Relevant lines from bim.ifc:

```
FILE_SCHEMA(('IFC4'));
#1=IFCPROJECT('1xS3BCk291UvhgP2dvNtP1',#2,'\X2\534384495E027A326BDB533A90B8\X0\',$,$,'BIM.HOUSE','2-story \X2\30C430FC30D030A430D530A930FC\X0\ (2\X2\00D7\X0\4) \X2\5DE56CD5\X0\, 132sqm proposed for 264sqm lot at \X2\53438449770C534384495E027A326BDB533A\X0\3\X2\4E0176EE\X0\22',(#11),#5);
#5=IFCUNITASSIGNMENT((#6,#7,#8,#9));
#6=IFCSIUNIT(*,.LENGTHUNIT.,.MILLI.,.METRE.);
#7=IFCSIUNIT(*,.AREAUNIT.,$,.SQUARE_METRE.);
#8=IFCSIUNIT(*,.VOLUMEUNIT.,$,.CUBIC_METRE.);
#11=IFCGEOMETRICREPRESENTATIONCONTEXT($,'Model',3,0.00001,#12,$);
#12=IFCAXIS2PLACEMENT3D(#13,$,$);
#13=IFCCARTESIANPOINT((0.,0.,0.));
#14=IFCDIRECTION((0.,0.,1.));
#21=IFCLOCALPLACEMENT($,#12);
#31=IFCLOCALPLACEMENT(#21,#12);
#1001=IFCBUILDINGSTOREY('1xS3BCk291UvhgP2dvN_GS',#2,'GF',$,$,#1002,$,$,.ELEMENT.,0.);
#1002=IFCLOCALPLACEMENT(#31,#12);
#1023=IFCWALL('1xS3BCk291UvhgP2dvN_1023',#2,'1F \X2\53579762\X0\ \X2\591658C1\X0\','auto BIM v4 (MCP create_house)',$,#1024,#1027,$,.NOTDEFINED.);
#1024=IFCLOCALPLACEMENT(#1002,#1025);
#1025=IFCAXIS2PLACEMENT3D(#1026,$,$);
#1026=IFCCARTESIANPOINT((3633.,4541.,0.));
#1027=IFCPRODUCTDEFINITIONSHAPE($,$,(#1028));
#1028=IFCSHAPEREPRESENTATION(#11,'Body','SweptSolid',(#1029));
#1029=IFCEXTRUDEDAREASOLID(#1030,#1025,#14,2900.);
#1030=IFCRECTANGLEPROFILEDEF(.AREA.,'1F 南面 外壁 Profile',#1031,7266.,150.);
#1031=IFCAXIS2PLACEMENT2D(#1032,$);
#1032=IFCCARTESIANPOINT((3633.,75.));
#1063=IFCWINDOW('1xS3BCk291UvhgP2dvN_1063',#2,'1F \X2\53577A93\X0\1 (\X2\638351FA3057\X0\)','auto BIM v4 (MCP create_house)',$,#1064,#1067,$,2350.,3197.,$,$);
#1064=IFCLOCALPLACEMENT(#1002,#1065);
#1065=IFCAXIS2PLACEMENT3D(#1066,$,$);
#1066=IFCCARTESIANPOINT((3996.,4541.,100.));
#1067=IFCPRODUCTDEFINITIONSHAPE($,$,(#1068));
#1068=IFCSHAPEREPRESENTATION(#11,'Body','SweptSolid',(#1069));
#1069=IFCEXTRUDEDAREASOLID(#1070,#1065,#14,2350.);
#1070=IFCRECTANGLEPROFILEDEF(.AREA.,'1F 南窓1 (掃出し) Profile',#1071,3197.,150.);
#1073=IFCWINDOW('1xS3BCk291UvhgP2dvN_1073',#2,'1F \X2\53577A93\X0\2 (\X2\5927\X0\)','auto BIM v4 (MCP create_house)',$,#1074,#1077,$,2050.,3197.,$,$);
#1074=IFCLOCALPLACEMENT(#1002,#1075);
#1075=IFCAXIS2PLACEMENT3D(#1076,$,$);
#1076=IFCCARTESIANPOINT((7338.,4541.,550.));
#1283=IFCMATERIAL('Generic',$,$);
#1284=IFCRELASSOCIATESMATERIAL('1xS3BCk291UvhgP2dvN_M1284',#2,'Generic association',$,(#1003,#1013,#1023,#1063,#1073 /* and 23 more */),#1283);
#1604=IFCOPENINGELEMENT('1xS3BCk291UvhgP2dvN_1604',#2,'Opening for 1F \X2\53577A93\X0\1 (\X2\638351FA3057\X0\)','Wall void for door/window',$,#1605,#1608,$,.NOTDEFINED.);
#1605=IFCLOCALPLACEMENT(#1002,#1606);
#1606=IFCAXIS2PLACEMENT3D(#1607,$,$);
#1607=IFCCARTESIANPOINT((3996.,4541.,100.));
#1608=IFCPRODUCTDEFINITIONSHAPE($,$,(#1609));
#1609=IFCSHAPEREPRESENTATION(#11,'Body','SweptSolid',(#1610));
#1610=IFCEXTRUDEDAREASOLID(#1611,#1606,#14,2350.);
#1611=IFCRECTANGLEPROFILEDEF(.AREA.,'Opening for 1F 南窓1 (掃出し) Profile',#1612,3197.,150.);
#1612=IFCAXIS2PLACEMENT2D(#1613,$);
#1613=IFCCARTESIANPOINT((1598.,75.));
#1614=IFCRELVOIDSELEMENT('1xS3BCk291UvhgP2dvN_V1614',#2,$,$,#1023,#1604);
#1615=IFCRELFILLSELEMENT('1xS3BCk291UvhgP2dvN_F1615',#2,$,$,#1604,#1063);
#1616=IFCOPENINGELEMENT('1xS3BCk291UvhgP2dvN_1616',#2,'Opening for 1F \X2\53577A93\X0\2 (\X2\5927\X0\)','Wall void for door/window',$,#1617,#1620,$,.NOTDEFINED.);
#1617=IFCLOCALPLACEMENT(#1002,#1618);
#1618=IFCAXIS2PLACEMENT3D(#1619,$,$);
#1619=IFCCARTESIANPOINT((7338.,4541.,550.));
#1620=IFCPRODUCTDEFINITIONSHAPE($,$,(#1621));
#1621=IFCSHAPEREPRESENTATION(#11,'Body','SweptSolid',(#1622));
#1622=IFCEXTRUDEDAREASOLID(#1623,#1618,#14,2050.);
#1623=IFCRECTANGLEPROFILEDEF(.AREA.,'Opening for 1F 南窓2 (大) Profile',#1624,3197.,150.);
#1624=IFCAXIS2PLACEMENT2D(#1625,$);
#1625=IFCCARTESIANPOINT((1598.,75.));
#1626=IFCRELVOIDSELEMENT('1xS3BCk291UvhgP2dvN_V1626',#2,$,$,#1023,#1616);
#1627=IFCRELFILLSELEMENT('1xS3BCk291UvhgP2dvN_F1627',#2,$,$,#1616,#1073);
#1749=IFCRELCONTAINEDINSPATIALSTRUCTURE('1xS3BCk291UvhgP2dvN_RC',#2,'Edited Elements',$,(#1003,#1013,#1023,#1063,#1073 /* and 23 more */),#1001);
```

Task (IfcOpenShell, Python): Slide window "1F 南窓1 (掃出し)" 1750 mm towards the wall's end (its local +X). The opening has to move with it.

```python
import ifcopenshell
import ifcopenshell.api.geometry
import ifcopenshell.util.placement

model = ifcopenshell.open("bim.ifc")

window = model.by_guid("1xS3BCk291UvhgP2dvN_1063")
opening = window.FillsVoids[0].RelatingOpeningElement
wall = opening.VoidsElements[0].RelatingBuildingElement

wall_matrix = ifcopenshell.util.placement.get_local_placement(wall.ObjectPlacement)
shift = wall_matrix[:3, 0] * 1750.0
before = ifcopenshell.util.placement.get_local_placement(window.ObjectPlacement)[:3, 3].copy()

# The window is not placed relative to its opening, so move both.
for product in (opening, window):
    matrix = ifcopenshell.util.placement.get_local_placement(product.ObjectPlacement)
    matrix[:3, 3] += shift
    ifcopenshell.api.geometry.edit_object_placement(model, product=product, matrix=matrix, is_si=False)

after = ifcopenshell.util.placement.get_local_placement(window.ObjectPlacement)[:3, 3]
print("window moved by", (after - before).round(3) + 0.0)

model.write("bim_edited.ifc")
```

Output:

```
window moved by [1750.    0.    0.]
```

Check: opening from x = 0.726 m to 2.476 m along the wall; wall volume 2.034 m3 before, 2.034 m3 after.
